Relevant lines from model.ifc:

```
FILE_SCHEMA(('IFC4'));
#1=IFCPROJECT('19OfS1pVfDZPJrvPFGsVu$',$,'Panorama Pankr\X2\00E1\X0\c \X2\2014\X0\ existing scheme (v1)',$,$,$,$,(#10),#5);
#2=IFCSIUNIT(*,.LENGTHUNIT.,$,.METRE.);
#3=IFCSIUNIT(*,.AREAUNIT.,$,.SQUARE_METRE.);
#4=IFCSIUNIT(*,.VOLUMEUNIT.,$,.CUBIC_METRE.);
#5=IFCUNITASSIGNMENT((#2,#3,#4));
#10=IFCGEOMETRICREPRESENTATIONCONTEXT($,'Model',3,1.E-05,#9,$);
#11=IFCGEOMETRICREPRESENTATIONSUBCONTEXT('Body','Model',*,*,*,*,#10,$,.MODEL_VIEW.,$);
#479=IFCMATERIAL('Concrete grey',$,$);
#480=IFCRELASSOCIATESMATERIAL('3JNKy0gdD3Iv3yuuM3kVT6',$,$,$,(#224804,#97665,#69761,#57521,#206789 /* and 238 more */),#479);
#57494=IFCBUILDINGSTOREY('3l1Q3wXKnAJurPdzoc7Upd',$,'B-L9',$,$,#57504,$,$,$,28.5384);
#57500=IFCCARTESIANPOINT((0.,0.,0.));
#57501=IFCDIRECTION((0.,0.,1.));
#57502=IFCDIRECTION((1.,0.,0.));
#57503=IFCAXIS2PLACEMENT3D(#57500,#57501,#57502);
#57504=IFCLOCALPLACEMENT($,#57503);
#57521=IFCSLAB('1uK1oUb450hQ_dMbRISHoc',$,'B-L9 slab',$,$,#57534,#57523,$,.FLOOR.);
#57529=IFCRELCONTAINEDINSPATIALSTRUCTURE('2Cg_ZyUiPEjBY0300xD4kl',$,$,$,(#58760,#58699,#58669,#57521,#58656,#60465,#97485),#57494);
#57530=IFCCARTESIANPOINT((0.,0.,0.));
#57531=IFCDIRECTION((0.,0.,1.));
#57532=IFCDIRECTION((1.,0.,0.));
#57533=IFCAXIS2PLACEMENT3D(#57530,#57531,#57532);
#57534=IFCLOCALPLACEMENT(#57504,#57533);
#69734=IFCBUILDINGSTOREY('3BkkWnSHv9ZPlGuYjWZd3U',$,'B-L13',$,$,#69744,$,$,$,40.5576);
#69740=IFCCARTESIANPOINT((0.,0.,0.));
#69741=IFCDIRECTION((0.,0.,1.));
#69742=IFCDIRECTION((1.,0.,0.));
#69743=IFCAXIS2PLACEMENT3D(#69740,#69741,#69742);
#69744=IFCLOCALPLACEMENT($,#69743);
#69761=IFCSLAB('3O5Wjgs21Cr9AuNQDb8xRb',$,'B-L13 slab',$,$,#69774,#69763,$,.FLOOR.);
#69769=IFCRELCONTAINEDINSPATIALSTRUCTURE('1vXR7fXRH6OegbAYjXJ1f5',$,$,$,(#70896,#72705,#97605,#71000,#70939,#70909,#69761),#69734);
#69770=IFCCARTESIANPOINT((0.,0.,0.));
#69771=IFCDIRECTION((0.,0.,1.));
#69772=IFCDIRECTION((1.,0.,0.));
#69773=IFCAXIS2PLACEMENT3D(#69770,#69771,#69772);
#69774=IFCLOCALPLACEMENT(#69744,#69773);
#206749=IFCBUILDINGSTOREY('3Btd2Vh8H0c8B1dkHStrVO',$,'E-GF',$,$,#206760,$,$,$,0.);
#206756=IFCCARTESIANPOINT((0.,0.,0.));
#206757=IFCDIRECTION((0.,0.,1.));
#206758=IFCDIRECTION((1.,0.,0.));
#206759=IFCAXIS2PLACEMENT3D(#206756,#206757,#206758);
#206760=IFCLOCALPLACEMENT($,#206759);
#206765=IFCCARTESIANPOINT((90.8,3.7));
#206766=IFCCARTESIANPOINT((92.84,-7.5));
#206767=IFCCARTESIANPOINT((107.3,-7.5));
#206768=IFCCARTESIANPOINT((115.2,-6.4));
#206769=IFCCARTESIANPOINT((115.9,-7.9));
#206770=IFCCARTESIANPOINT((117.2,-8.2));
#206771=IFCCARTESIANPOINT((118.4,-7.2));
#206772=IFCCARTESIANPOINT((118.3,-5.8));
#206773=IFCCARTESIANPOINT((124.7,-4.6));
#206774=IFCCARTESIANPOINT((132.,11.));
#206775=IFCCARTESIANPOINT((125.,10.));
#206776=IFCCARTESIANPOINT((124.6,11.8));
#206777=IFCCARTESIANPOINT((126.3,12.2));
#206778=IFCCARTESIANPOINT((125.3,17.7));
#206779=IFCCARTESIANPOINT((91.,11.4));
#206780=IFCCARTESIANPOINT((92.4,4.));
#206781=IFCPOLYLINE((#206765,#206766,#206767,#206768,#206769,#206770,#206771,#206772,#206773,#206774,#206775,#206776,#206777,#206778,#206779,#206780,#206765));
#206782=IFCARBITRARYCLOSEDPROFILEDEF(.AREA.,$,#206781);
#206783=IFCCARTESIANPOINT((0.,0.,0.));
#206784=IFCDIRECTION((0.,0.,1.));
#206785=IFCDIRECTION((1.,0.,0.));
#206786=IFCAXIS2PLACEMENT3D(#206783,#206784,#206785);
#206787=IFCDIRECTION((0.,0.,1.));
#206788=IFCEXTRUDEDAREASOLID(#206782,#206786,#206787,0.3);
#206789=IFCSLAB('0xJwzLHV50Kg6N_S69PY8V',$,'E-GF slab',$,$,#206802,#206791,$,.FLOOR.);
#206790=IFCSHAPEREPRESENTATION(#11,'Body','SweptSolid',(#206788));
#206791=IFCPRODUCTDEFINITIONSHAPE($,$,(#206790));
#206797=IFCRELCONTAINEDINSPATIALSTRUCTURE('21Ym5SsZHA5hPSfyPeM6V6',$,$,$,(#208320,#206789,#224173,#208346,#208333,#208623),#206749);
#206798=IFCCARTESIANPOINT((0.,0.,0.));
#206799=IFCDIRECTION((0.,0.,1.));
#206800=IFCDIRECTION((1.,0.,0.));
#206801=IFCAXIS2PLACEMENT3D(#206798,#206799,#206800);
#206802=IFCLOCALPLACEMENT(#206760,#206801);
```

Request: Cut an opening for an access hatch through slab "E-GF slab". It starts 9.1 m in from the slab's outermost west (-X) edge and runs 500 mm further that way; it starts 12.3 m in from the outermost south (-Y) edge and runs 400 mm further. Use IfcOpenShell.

```python
import numpy as np
import ifcopenshell
import ifcopenshell.api.feature
import ifcopenshell.api.geometry
import ifcopenshell.api.root
import ifcopenshell.geom
import ifcopenshell.util.placement
import ifcopenshell.util.representation
import ifcopenshell.util.shape
import ifcopenshell.util.unit

model = ifcopenshell.open("model.ifc")
unit_scale = ifcopenshell.util.unit.calculate_unit_scale(model)
settings = ifcopenshell.geom.settings()


def volume(element):
    """Net volume in cubic metres, openings subtracted."""
    shape = ifcopenshell.geom.create_shape(settings, element)
    return ifcopenshell.util.shape.get_volume(shape.geometry)


slab = model.by_guid("0xJwzLHV50Kg6N_S69PY8V")
before = volume(slab)

# Extent in the slab's own axes, in metres. The edges named are its -X and -Y sides.
slab_shape = ifcopenshell.geom.create_shape(settings, slab)
vertices = ifcopenshell.util.shape.get_vertices(slab_shape.geometry)
x_min, y_min, bottom = vertices.min(axis=0)
top = vertices[:, 2].max()

opening = ifcopenshell.api.root.create_entity(model, ifc_class="IfcOpeningElement", name="Access hatch opening", predefined_type="OPENING")
context = ifcopenshell.util.representation.get_context(model, "Model", "Body", "MODEL_VIEW")
width, depth = 0.5, 0.4
outline = [(0.0, 0.0), (width, 0.0), (width, depth), (0.0, depth), (0.0, 0.0)]
# Overshoot both faces by 50 mm so the cut is clean.
shape = ifcopenshell.api.geometry.add_slab_representation(
    model, context=context, depth=top - bottom + 0.1, polyline=outline
)
ifcopenshell.api.geometry.assign_representation(model, product=opening, representation=shape)

matrix = ifcopenshell.util.placement.get_local_placement(slab.ObjectPlacement)
matrix[:, 3] = matrix @ np.append(np.array([x_min + 9.1, y_min + 12.3, bottom - 0.05]) / unit_scale, 1.0)
ifcopenshell.api.geometry.edit_object_placement(model, product=opening, matrix=matrix, is_si=False)
ifcopenshell.api.feature.add_feature(model, feature=opening, element=slab)

after = volume(slab)

print(f"slab volume {before:.3f} -> {after:.3f} m3")

model.write("model_edited.ifc")
```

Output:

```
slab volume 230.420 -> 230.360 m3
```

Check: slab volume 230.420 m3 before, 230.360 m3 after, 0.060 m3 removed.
